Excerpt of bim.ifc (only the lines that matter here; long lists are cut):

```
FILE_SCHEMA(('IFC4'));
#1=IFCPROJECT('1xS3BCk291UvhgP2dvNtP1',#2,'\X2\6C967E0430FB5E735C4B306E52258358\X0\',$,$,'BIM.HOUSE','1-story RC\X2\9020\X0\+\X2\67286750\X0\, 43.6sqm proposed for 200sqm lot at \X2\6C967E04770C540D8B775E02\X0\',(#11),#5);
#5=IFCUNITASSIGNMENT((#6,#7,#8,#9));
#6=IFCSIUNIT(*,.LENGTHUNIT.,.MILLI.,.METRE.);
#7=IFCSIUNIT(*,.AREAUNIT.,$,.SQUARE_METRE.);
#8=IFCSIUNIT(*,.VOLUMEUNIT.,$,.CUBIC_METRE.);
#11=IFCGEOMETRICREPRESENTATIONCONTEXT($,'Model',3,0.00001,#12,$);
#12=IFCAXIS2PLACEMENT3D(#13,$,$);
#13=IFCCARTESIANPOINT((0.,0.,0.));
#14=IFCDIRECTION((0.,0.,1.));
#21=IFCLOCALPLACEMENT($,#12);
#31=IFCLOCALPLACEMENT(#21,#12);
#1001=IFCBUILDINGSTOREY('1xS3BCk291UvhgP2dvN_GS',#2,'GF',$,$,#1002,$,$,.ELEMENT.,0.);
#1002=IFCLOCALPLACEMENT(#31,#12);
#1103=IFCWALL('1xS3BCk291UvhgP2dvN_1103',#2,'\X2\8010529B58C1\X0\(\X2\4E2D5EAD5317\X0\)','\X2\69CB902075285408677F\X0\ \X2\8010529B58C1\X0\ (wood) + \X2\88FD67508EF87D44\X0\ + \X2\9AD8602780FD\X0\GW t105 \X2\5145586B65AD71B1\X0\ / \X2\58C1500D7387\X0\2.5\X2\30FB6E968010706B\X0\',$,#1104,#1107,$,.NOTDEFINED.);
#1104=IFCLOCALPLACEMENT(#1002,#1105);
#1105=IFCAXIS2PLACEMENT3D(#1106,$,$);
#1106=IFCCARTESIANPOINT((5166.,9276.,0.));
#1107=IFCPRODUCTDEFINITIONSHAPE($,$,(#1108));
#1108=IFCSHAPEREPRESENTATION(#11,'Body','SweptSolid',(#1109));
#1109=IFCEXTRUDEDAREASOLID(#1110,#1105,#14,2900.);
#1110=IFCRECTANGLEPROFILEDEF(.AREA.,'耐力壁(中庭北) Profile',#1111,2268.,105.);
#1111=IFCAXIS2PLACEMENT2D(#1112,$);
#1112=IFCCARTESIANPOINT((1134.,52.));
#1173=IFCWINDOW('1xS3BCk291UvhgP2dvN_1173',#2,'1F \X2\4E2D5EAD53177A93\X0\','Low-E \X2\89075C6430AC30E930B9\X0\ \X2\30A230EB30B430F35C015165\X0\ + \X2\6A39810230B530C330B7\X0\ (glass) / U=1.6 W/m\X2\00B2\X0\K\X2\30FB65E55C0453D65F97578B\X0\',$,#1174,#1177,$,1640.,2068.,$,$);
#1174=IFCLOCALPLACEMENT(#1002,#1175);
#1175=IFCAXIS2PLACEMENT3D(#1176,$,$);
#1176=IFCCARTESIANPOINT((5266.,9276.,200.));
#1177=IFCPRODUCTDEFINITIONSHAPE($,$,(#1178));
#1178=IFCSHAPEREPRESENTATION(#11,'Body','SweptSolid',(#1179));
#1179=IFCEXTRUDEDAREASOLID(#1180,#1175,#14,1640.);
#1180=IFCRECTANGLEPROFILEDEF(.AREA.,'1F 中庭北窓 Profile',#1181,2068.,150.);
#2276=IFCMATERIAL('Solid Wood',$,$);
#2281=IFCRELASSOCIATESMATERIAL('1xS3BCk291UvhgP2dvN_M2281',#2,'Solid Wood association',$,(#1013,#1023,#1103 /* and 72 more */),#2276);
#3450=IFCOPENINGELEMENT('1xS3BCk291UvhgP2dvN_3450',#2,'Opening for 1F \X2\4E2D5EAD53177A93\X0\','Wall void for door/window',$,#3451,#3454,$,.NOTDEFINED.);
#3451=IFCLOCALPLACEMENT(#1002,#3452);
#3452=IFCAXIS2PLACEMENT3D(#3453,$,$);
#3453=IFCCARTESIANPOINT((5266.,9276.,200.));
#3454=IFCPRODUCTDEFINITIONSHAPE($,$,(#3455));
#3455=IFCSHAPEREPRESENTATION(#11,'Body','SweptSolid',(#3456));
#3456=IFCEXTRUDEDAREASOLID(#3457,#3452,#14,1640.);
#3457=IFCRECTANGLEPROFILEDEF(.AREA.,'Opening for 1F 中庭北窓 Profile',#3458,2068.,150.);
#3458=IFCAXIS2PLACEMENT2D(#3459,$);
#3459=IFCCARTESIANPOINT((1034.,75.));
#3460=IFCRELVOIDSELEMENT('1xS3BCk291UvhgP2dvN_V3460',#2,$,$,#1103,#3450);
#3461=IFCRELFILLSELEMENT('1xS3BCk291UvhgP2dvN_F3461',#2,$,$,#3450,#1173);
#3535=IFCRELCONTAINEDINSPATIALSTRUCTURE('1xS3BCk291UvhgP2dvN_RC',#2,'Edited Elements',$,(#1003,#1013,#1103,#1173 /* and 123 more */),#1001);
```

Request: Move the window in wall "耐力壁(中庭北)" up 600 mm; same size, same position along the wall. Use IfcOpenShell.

```python
import numpy as np
import ifcopenshell
import ifcopenshell.api.geometry
import ifcopenshell.util.placement
import ifcopenshell.util.unit

model = ifcopenshell.open("bim.ifc")
unit_scale = ifcopenshell.util.unit.calculate_unit_scale(model)

window = model.by_guid("1xS3BCk291UvhgP2dvN_1173")
opening = window.FillsVoids[0].RelatingOpeningElement
dz = 0.6 / unit_scale

shift = np.array([0.0, 0.0, dz])
# The window is not placed relative to its opening, so move both.
for product in (opening, window):
    matrix = ifcopenshell.util.placement.get_local_placement(product.ObjectPlacement)
    matrix[:3, 3] += shift
    ifcopenshell.api.geometry.edit_object_placement(model, product=product, matrix=matrix, is_si=False)

print(f"moved by {dz * unit_scale:+.3f} m")

model.write("bim-out.ifc")
```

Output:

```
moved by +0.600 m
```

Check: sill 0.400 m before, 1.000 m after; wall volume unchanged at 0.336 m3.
